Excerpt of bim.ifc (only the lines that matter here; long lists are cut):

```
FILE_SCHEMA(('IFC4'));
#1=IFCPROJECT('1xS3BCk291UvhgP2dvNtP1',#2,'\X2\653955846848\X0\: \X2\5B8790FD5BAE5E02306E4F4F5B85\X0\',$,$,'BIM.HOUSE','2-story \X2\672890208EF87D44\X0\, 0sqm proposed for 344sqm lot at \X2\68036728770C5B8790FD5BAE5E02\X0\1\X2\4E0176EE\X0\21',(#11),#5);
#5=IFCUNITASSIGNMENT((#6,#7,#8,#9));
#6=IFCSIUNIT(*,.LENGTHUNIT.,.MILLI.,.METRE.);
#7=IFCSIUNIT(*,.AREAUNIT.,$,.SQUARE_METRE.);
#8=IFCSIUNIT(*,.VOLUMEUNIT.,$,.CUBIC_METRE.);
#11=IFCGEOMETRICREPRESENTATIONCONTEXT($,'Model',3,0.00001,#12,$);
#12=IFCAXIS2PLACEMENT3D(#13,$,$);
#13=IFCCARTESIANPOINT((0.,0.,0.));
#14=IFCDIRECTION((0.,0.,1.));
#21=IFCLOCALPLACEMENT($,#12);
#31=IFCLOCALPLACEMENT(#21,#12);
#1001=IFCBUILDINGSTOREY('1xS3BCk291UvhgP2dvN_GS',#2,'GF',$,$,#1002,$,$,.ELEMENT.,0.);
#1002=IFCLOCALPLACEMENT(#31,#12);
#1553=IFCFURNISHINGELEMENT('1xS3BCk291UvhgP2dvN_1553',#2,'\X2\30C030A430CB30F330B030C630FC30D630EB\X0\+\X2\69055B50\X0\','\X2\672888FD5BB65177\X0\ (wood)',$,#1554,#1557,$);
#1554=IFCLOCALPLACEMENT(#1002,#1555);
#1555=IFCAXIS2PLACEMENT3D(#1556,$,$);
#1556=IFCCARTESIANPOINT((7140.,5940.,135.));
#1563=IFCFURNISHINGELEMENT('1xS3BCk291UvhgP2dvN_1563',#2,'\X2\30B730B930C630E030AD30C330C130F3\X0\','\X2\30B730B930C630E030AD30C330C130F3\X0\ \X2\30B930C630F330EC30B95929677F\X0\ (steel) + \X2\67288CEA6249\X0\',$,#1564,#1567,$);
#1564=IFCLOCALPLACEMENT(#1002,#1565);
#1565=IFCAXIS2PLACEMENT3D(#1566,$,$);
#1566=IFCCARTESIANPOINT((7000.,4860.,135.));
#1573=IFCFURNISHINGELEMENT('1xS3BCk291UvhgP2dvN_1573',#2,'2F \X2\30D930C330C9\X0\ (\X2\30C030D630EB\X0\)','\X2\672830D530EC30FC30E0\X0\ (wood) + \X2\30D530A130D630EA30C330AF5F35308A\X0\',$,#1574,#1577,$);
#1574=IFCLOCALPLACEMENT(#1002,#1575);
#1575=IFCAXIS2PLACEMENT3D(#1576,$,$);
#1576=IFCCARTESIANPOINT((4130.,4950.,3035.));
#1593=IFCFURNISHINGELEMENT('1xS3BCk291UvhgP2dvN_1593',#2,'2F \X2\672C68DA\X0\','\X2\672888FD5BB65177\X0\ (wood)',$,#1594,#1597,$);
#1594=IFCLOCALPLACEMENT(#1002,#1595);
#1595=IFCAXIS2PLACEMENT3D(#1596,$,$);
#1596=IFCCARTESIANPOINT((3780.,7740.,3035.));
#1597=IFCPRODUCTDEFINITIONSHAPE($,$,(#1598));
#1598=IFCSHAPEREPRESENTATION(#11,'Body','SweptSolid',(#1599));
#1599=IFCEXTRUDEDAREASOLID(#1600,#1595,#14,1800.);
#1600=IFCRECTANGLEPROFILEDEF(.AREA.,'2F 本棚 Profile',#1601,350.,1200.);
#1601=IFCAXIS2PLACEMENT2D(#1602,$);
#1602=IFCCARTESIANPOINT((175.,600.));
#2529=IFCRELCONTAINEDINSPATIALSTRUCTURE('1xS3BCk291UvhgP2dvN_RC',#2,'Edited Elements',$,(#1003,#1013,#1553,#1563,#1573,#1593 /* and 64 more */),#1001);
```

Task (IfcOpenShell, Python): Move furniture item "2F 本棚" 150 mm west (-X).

```python
import ifcopenshell
import ifcopenshell.api.geometry
import ifcopenshell.util.placement
import ifcopenshell.util.unit

model = ifcopenshell.open("bim.ifc")
unit_scale = ifcopenshell.util.unit.calculate_unit_scale(model)

item = model.by_id(1593)
matrix = ifcopenshell.util.placement.get_local_placement(item.ObjectPlacement)
matrix[0, 3] -= 0.15 / unit_scale
ifcopenshell.api.geometry.edit_object_placement(model, product=item, matrix=matrix, is_si=False)

print(ifcopenshell.util.placement.get_local_placement(item.ObjectPlacement).round(3) + 0.0)

model.write("bim-out.ifc")
```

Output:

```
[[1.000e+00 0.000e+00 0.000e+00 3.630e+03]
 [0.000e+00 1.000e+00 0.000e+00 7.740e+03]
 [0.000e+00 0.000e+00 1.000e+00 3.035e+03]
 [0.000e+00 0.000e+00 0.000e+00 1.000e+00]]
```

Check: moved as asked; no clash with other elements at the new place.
